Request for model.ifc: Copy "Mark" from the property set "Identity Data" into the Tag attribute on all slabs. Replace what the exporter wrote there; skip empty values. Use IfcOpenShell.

First a look at what the model holds.

```python
import ifcopenshell
import ifcopenshell.util.element

model = ifcopenshell.open("model.ifc")
print(model.schema)
slabs = model.by_type("IfcSlab")
print(len(slabs), "slabs")
for e in slabs[:8]:
    source = ifcopenshell.util.element.get_pset(e, "Identity Data", "Mark")
    target = e.Tag
    print(e.id(), repr(source), repr(target), sep=" | ")
```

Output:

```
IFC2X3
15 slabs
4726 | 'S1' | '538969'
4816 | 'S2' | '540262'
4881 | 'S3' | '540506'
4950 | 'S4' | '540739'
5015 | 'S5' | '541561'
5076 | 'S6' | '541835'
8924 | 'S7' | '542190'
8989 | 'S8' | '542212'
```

```python
import ifcopenshell
import ifcopenshell.util.element

model = ifcopenshell.open("model.ifc")

count = 0
for e in model.by_type("IfcSlab"):
    value = ifcopenshell.util.element.get_pset(e, "Identity Data", "Mark")
    current = e.Tag
    if not value or not value.strip() or current == value:
        continue
    e.Tag = value
    count += 1

print(count, "slabs updated")

model.write("model-out.ifc")
```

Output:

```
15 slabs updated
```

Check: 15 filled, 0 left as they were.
